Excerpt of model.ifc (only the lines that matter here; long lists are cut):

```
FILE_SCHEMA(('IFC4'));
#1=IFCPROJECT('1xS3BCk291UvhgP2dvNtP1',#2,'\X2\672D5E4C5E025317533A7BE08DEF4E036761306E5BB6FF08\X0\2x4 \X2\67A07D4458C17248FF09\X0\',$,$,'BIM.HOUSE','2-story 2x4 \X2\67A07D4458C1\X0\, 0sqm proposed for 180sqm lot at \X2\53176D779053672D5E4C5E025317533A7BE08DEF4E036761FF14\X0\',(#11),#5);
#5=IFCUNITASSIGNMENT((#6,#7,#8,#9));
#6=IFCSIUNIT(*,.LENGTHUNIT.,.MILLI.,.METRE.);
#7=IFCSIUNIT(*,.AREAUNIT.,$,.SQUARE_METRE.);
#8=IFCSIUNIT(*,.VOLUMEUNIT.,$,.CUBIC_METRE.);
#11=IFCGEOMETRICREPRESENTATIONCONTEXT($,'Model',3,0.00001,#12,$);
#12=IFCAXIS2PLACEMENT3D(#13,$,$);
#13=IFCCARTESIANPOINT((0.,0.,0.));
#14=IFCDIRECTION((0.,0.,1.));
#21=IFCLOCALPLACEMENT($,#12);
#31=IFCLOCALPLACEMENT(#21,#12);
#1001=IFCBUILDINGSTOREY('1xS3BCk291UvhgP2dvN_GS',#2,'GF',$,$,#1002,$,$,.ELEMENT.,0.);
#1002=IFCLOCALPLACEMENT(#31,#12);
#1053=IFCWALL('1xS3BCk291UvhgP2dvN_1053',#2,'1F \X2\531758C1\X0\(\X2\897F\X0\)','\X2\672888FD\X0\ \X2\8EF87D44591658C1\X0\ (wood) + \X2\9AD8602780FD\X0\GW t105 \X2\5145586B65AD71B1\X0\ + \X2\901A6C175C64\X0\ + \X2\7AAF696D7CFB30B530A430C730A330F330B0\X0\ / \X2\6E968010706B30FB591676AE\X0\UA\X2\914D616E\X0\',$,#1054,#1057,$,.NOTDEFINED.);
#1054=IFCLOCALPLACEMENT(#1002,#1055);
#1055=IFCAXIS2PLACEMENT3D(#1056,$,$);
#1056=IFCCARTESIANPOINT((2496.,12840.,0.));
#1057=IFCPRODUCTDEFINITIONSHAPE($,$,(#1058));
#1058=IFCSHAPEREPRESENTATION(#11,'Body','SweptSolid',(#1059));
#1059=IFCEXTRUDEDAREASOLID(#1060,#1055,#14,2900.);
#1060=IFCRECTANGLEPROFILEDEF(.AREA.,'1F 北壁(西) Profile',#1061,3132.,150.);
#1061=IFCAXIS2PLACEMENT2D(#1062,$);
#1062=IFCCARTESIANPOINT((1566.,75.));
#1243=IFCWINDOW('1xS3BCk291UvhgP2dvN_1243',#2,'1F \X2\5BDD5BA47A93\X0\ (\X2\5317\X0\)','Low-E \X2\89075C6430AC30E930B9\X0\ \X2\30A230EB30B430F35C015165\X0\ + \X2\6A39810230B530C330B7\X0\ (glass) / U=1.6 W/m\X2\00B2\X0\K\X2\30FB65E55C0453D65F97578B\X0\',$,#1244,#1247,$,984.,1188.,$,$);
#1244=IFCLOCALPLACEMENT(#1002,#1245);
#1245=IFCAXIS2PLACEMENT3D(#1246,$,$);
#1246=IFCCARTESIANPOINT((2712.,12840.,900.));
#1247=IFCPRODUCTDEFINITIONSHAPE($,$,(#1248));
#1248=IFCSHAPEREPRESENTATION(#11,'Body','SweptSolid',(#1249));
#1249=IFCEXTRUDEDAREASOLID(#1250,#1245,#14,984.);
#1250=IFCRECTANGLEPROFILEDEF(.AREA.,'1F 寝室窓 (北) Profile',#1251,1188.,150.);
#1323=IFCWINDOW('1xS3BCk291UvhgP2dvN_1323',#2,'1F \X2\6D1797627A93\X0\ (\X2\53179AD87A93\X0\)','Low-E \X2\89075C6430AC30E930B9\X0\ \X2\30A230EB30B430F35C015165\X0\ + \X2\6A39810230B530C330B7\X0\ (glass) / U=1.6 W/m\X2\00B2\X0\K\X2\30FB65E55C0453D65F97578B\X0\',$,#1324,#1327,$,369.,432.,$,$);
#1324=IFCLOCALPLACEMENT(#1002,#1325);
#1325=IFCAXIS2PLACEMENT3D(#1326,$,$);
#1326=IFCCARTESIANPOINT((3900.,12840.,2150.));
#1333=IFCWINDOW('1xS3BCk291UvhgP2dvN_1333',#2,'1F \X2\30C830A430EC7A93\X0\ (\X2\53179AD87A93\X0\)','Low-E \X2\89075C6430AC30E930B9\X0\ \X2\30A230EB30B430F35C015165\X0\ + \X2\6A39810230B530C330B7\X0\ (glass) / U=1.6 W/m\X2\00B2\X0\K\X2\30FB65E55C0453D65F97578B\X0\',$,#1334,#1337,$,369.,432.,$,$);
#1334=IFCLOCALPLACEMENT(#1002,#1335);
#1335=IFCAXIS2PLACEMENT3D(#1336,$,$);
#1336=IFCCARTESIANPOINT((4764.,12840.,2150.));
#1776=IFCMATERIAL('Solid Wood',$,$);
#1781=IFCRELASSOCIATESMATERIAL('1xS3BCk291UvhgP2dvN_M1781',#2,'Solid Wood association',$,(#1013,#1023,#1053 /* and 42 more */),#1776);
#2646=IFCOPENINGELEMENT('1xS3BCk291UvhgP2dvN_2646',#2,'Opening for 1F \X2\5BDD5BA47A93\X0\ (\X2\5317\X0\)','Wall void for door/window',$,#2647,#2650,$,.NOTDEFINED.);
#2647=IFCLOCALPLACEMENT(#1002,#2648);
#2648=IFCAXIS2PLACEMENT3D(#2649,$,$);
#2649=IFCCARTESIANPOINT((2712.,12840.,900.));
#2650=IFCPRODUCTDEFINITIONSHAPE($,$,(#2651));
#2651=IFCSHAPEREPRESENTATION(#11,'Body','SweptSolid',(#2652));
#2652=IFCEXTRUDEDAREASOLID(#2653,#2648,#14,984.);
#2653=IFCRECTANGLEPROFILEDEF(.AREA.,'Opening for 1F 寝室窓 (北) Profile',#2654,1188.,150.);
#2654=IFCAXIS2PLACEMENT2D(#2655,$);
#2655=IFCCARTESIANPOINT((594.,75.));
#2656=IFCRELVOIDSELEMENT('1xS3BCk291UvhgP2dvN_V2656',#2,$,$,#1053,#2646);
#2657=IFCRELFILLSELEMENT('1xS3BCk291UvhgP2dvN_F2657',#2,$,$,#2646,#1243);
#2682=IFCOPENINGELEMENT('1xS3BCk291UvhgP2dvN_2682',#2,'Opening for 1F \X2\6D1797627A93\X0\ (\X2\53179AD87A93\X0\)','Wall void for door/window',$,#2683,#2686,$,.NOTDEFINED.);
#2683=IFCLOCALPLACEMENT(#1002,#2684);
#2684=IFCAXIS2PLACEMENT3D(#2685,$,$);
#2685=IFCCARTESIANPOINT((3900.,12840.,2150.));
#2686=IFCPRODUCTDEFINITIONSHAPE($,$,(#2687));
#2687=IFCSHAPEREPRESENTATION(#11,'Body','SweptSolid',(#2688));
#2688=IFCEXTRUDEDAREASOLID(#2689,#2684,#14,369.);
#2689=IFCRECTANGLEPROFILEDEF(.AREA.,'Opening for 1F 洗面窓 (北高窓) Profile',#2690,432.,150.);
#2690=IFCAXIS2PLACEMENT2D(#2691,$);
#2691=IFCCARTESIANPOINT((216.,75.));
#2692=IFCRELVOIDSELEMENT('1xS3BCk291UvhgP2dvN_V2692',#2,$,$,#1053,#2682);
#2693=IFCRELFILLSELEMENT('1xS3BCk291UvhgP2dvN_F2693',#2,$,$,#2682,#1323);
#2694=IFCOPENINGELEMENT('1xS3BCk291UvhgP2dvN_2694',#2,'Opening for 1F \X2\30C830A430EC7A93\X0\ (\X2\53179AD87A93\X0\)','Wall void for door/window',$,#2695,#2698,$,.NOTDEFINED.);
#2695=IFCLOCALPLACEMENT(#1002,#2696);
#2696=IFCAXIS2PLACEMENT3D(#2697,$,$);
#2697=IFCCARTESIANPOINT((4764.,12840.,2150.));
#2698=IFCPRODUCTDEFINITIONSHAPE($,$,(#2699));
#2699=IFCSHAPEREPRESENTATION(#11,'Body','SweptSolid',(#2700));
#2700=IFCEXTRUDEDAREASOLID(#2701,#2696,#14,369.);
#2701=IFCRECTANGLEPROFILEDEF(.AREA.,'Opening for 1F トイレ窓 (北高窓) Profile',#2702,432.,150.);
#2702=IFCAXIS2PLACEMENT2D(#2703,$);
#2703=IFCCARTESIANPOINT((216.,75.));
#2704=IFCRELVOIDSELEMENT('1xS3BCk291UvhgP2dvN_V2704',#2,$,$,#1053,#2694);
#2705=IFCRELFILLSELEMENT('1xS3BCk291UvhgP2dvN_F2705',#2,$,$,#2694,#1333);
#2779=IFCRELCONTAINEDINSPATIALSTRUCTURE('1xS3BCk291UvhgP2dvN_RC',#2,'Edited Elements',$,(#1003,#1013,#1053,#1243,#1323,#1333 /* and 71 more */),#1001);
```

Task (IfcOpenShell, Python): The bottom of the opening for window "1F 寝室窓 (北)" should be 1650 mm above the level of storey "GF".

```python
import numpy as np
import ifcopenshell
import ifcopenshell.api.geometry
import ifcopenshell.geom
import ifcopenshell.util.element
import ifcopenshell.util.placement
import ifcopenshell.util.shape
import ifcopenshell.util.unit

model = ifcopenshell.open("model.ifc")
unit_scale = ifcopenshell.util.unit.calculate_unit_scale(model)

window = model.by_guid("1xS3BCk291UvhgP2dvN_1243")
opening = window.FillsVoids[0].RelatingOpeningElement
storey = ifcopenshell.util.element.get_container(window, ifc_class="IfcBuildingStorey")
level = ifcopenshell.util.placement.get_local_placement(storey.ObjectPlacement)[2, 3]

# The opening's origin need not be at the sill, so measure its lowest point.
shape = ifcopenshell.geom.create_shape(ifcopenshell.geom.settings(), opening)
bottom = ifcopenshell.util.shape.get_shape_bottom_elevation(shape, shape.geometry) / unit_scale
dz = level + 1650.0 - bottom

shift = np.array([0.0, 0.0, dz])
# The window is not placed relative to its opening, so move both.
for product in (opening, window):
    matrix = ifcopenshell.util.placement.get_local_placement(product.ObjectPlacement)
    matrix[:3, 3] += shift
    ifcopenshell.api.geometry.edit_object_placement(model, product=product, matrix=matrix, is_si=False)

print(f"moved by {dz * unit_scale:+.3f} m")

model.write("model_updated.ifc")
```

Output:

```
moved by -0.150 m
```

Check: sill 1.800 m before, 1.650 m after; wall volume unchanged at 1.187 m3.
